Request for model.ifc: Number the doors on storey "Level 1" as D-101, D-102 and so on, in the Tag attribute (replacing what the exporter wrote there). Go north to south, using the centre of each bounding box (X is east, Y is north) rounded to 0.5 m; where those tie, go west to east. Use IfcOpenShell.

First a look at what the model holds.

```python
import ifcopenshell
import ifcopenshell.util.element
import ifcopenshell.util.placement

model = ifcopenshell.open("model.ifc")
print(model.schema)
storey = next(s for s in model.by_type("IfcBuildingStorey") if s.Name == "Level 1")
doors = [e for e in ifcopenshell.util.element.get_decomposition(storey) if e.is_a("IfcDoor")]
for e in sorted(doors, key=lambda e: e.id()):
    origin = ifcopenshell.util.placement.get_local_placement(e.ObjectPlacement)[:3, 3]
    print(e.id(), e.Tag, e.Name, origin.round(2) + 0.0, sep=" | ")
```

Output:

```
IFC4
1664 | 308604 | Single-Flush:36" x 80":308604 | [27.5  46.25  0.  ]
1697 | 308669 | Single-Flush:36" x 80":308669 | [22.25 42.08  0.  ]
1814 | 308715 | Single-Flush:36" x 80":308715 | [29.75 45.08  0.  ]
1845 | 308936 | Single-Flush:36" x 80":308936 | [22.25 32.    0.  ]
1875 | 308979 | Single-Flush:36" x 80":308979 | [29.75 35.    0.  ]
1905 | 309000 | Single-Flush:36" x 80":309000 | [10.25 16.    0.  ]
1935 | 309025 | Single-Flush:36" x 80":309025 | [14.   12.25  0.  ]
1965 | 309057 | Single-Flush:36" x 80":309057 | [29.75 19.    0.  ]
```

```python
import ifcopenshell
import ifcopenshell.geom
import ifcopenshell.util.element
import ifcopenshell.util.shape

model = ifcopenshell.open("model.ifc")
settings = ifcopenshell.geom.settings()
settings.set("use-world-coords", True)


def centre(element):
    shape = ifcopenshell.geom.create_shape(settings, element)
    return ifcopenshell.util.shape.get_bbox_centroid(shape.geometry)


storey = next(s for s in model.by_type("IfcBuildingStorey") if s.Name == "Level 1")
doors = [e for e in ifcopenshell.util.element.get_decomposition(storey) if e.is_a("IfcDoor")]

# Insertion points can sit at a corner or the storey origin, so sort by the geometry (in metres).
centres = {e: centre(e) for e in doors}
doors.sort(key=lambda e: (-round(centres[e][1] / 0.5), centres[e][0]))

for i, e in enumerate(doors, start=1):
    number = f"D-1{i:02d}"
    e.Tag = number
    print(e.id(), number)

model.write("model_rev.ifc")
```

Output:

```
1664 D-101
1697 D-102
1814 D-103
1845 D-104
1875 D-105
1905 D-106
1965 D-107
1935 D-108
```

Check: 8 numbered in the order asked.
